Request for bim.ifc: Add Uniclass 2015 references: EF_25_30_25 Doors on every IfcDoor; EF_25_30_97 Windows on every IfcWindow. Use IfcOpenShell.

First a look at what the model holds.

```python
import ifcopenshell

model = ifcopenshell.open("bim.ifc")
print(model.schema)
print("classifications:", [c.Name for c in model.by_type("IfcClassification")])
for ifc_class in ("IfcDoor", "IfcRoof", "IfcStair", "IfcWall", "IfcWindow"):
    print(ifc_class, len(model.by_type(ifc_class)))
```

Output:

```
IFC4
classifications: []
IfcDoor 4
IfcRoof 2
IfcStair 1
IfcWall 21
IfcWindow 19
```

```python
import ifcopenshell
import ifcopenshell.api.classification

model = ifcopenshell.open("bim.ifc")

system = ifcopenshell.api.classification.add_classification(model, classification="Uniclass 2015")

codes = {
    "IfcDoor": ("EF_25_30_25", "Doors"),
    "IfcWindow": ("EF_25_30_97", "Windows"),
}
for ifc_class, (code, name) in codes.items():
    products = model.by_type(ifc_class)
    ifcopenshell.api.classification.add_reference(
        model, products=products, classification=system, identification=code, name=name
    )
    print(code, len(products))

model.write("bim_v2.ifc")
```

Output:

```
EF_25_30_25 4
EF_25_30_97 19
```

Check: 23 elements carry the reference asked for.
